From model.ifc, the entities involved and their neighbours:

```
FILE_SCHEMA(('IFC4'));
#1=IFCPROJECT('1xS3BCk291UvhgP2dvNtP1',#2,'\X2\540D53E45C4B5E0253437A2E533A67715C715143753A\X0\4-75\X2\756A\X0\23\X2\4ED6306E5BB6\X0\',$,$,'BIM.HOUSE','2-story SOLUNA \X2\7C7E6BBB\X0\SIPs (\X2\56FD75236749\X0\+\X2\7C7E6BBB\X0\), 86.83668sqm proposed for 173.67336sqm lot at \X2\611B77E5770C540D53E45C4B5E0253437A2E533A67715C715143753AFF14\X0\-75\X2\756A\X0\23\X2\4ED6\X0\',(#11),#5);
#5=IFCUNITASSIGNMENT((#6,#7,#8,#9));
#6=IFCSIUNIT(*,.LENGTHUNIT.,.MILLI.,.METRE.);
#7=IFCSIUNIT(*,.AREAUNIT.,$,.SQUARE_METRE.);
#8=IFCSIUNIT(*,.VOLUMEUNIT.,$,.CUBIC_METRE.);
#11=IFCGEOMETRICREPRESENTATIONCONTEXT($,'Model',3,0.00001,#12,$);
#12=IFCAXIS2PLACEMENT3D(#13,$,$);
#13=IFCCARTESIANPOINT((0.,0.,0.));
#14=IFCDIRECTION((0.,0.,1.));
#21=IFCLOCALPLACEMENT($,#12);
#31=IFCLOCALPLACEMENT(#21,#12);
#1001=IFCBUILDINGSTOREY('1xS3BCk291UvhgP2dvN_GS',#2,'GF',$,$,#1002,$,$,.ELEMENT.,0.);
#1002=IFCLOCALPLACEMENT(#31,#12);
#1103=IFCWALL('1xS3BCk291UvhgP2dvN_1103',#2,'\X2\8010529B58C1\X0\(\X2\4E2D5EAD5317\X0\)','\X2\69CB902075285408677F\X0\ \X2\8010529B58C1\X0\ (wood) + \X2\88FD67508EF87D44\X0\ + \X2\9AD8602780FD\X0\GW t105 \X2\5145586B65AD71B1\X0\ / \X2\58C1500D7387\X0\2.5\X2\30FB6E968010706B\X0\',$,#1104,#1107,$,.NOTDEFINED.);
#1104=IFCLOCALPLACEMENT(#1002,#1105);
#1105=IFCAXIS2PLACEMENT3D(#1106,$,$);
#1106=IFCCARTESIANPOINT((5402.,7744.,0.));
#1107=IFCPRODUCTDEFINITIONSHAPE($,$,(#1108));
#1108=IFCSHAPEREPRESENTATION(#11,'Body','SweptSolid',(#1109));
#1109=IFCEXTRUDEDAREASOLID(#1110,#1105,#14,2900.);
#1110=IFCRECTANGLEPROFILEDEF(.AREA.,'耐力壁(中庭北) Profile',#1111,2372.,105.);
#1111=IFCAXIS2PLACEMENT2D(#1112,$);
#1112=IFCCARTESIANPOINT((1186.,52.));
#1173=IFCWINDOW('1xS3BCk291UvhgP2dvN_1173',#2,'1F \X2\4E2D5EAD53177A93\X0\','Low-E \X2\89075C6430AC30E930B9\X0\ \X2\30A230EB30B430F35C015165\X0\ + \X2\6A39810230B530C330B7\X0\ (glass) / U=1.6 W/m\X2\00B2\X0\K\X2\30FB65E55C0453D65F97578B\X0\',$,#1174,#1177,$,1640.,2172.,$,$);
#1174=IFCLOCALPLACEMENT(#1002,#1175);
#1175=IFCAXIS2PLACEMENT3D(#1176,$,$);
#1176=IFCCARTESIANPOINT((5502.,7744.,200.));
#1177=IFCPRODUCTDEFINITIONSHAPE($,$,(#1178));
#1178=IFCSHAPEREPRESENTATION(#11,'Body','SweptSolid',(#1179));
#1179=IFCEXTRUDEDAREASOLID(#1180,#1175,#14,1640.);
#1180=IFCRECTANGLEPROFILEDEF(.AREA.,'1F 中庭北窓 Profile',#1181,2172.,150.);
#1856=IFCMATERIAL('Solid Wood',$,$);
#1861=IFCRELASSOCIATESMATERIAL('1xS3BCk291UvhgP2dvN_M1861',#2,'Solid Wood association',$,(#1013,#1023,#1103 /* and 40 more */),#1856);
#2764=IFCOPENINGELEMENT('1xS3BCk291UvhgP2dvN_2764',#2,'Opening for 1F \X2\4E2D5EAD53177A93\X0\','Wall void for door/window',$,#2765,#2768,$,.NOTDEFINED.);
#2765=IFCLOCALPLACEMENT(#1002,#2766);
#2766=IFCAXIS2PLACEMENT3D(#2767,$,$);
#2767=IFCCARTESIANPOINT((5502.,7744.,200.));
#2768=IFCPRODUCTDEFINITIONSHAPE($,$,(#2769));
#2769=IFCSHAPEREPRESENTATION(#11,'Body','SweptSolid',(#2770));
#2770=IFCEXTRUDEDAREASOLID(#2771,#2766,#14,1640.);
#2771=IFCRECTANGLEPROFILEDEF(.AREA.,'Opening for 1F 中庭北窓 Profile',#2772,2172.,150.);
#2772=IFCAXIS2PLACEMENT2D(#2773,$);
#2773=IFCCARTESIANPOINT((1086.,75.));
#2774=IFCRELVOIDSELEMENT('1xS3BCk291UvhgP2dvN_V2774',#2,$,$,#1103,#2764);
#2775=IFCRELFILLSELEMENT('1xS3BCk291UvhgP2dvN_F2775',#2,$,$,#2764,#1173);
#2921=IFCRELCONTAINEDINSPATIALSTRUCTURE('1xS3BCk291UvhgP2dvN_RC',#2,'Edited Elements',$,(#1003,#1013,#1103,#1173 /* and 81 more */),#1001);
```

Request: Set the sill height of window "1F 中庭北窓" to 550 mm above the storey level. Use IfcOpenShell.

```python
import numpy as np
import ifcopenshell
import ifcopenshell.api.geometry
import ifcopenshell.geom
import ifcopenshell.util.element
import ifcopenshell.util.placement
import ifcopenshell.util.shape
import ifcopenshell.util.unit

model = ifcopenshell.open("model.ifc")
unit_scale = ifcopenshell.util.unit.calculate_unit_scale(model)

window = model.by_guid("1xS3BCk291UvhgP2dvN_1173")
opening = window.FillsVoids[0].RelatingOpeningElement
storey = ifcopenshell.util.element.get_container(window, ifc_class="IfcBuildingStorey")
level = ifcopenshell.util.placement.get_local_placement(storey.ObjectPlacement)[2, 3]

# The opening's origin need not be at the sill, so measure its lowest point.
shape = ifcopenshell.geom.create_shape(ifcopenshell.geom.settings(), opening)
bottom = ifcopenshell.util.shape.get_shape_bottom_elevation(shape, shape.geometry) / unit_scale
dz = level + 0.55 / unit_scale - bottom

shift = np.array([0.0, 0.0, dz])
# The window is not placed relative to its opening, so move both.
for product in (opening, window):
    matrix = ifcopenshell.util.placement.get_local_placement(product.ObjectPlacement)
    matrix[:3, 3] += shift
    ifcopenshell.api.geometry.edit_object_placement(model, product=product, matrix=matrix, is_si=False)

print(f"moved by {dz * unit_scale:+.3f} m")

model.write("model-out.ifc")
```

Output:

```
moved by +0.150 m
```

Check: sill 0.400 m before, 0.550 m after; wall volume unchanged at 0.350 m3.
